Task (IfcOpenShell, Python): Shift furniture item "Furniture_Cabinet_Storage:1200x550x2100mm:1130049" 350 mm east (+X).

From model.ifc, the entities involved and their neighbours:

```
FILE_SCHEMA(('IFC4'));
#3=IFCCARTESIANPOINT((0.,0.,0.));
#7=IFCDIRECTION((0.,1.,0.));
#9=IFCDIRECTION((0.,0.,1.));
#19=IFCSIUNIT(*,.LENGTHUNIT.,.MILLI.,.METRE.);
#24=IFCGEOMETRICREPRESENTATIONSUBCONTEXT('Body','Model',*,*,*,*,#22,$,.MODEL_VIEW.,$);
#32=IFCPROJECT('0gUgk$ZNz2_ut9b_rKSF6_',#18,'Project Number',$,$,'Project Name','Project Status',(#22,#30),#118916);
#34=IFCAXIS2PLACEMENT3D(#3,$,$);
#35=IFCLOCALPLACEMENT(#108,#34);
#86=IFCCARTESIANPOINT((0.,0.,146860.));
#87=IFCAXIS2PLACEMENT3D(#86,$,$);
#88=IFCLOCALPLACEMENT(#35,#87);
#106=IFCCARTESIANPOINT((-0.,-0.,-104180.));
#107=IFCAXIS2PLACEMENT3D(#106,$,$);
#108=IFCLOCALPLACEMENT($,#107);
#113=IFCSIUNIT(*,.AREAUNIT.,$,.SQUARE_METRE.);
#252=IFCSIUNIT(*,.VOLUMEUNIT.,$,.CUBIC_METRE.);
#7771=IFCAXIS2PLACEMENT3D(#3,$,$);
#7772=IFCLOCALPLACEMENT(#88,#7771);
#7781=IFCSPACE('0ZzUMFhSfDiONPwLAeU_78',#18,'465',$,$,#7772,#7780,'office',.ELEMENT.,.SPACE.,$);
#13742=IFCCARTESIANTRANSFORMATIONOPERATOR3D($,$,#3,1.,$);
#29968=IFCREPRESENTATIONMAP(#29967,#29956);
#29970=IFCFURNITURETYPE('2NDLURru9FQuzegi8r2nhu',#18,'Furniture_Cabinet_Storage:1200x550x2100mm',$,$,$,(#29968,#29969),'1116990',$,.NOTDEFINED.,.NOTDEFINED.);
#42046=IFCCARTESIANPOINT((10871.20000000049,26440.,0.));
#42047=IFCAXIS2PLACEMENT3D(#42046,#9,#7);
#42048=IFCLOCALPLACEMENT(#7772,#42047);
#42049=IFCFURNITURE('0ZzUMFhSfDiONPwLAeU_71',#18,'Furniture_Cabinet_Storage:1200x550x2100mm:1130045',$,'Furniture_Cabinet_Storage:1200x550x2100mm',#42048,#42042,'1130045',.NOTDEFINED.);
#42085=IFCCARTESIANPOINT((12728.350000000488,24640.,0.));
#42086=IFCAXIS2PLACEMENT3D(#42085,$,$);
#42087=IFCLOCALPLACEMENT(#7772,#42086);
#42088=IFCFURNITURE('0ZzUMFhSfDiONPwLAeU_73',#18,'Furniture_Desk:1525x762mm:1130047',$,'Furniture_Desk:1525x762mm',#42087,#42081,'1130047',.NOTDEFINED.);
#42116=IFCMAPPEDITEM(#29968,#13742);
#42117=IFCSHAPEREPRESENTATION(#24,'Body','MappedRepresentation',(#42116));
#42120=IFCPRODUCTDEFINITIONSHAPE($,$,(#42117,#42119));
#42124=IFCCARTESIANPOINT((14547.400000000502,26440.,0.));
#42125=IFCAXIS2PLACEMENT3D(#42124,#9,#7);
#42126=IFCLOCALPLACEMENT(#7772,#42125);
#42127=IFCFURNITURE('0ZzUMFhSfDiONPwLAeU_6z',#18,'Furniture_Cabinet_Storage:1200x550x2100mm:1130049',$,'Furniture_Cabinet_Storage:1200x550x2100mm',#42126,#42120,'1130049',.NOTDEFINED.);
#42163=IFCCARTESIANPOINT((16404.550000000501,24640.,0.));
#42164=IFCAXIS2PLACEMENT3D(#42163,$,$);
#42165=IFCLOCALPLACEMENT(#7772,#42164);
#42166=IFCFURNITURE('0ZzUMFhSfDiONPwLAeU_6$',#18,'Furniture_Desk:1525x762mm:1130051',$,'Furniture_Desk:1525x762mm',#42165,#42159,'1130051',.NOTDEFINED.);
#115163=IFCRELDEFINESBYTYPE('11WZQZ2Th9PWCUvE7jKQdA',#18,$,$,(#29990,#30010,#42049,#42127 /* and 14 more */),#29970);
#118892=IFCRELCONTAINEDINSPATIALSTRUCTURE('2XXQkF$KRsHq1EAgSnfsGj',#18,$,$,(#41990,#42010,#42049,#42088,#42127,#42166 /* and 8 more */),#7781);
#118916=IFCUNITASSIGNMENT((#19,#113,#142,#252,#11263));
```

```python
import ifcopenshell
import ifcopenshell.api.geometry
import ifcopenshell.util.placement
import ifcopenshell.util.unit

model = ifcopenshell.open("model.ifc")
unit_scale = ifcopenshell.util.unit.calculate_unit_scale(model)

item = model.by_guid("0ZzUMFhSfDiONPwLAeU_6z")
matrix = ifcopenshell.util.placement.get_local_placement(item.ObjectPlacement)
matrix[0, 3] += 0.35 / unit_scale
ifcopenshell.api.geometry.edit_object_placement(model, product=item, matrix=matrix, is_si=False)

print(ifcopenshell.util.placement.get_local_placement(item.ObjectPlacement).round(3) + 0.0)

model.write("model_rev.ifc")
```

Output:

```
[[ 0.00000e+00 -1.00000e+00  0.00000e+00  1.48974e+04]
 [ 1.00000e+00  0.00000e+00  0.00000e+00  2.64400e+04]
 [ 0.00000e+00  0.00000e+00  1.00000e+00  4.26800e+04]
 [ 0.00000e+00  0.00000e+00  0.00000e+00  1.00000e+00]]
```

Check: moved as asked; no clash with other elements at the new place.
